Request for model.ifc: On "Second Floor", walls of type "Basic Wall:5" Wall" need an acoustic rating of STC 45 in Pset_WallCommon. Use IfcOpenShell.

First a look at what the model holds.

```python
import ifcopenshell
import ifcopenshell.util.element

model = ifcopenshell.open("model.ifc")
print(model.schema)
storey = next(s for s in model.by_type("IfcBuildingStorey") if s.Name == "Second Floor")
walls = [e for e in ifcopenshell.util.element.get_decomposition(storey) if e.is_a("IfcWall")]
seen = {}
for e in walls:
    element_type = ifcopenshell.util.element.get_type(e)
    key = (element_type.Name if element_type != e and element_type else None, ifcopenshell.util.element.get_pset(e, "Pset_WallCommon", "AcousticRating"))
    seen[key] = seen.get(key, 0) + 1
for (name, value), count in sorted(seen.items(), key=str):
    print(count, "x", name, "|", value)
```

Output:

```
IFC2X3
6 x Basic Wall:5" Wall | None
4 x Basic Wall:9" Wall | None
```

```python
import ifcopenshell
import ifcopenshell.api.pset
import ifcopenshell.util.element

model = ifcopenshell.open("model.ifc")

storey = next(s for s in model.by_type("IfcBuildingStorey") if s.Name == "Second Floor")
walls = [e for e in ifcopenshell.util.element.get_decomposition(storey) if e.is_a("IfcWall")]

count = 0
for e in walls:
    element_type = ifcopenshell.util.element.get_type(e)
    if element_type in (None, e) or element_type.Name != 'Basic Wall:5" Wall':
        continue
    # add_pset returns the element's existing set when there is one.
    pset = ifcopenshell.api.pset.add_pset(model, product=e, name="Pset_WallCommon")
    ifcopenshell.api.pset.edit_pset(model, pset=pset, properties={"AcousticRating": "STC 45"})
    count += 1

print(count, "walls updated")

model.write("model-out.ifc")
```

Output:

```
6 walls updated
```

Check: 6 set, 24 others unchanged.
